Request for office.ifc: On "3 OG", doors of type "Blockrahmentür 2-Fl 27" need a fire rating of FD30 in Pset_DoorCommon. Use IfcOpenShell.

First a look at what the model holds.

```python
import ifcopenshell
import ifcopenshell.util.element

model = ifcopenshell.open("office.ifc")
print(model.schema)
storey = next(s for s in model.by_type("IfcBuildingStorey") if s.Name == "3 OG")
doors = [e for e in ifcopenshell.util.element.get_decomposition(storey) if e.is_a("IfcDoor")]
seen = {}
for e in doors:
    element_type = ifcopenshell.util.element.get_type(e)
    key = (element_type.Name if element_type != e and element_type else None, ifcopenshell.util.element.get_pset(e, "Pset_DoorCommon", "FireRating"))
    seen[key] = seen.get(key, 0) + 1
for (name, value), count in sorted(seen.items(), key=str):
    print(count, "x", name, "|", value)
```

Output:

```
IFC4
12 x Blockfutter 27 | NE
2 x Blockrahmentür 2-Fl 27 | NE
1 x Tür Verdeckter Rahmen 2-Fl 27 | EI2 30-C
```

```python
import ifcopenshell
import ifcopenshell.api.pset
import ifcopenshell.util.element

model = ifcopenshell.open("office.ifc")

storey = next(s for s in model.by_type("IfcBuildingStorey") if s.Name == "3 OG")
doors = [e for e in ifcopenshell.util.element.get_decomposition(storey) if e.is_a("IfcDoor")]

count = 0
for e in doors:
    element_type = ifcopenshell.util.element.get_type(e)
    if element_type in (None, e) or element_type.Name != "Blockrahmentür 2-Fl 27":
        continue
    # add_pset returns the element's existing set when there is one.
    pset = ifcopenshell.api.pset.add_pset(model, product=e, name="Pset_DoorCommon")
    ifcopenshell.api.pset.edit_pset(model, pset=pset, properties={"FireRating": "FD30"})
    count += 1

print(count, "doors updated")

model.write("office-out.ifc")
```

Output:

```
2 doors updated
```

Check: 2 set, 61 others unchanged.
